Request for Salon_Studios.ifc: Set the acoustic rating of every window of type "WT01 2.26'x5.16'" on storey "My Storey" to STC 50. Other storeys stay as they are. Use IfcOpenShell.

First a look at what the model holds.

```python
import ifcopenshell
import ifcopenshell.util.element

model = ifcopenshell.open("Salon_Studios.ifc")
print(model.schema)
storey = next(s for s in model.by_type("IfcBuildingStorey") if s.Name == "My Storey")
windows = [e for e in ifcopenshell.util.element.get_decomposition(storey) if e.is_a("IfcWindow")]
seen = {}
for e in windows:
    element_type = ifcopenshell.util.element.get_type(e)
    key = (element_type.Name if element_type != e and element_type else None, ifcopenshell.util.element.get_pset(e, "Pset_WindowCommon", "AcousticRating"))
    seen[key] = seen.get(key, 0) + 1
for (name, value), count in sorted(seen.items(), key=str):
    print(count, "x", name, "|", value)
```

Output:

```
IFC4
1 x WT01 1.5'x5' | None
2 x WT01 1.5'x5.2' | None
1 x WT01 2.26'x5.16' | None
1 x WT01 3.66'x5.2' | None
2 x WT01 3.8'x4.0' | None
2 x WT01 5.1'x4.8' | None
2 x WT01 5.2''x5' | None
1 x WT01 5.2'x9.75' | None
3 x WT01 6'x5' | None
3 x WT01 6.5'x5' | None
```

```python
import ifcopenshell
import ifcopenshell.api.pset
import ifcopenshell.util.element

model = ifcopenshell.open("Salon_Studios.ifc")

storey = next(s for s in model.by_type("IfcBuildingStorey") if s.Name == "My Storey")
windows = [e for e in ifcopenshell.util.element.get_decomposition(storey) if e.is_a("IfcWindow")]

count = 0
for e in windows:
    element_type = ifcopenshell.util.element.get_type(e)
    if element_type in (None, e) or element_type.Name != "WT01 2.26'x5.16'":
        continue
    # add_pset returns the element's existing set when there is one.
    pset = ifcopenshell.api.pset.add_pset(model, product=e, name="Pset_WindowCommon")
    ifcopenshell.api.pset.edit_pset(model, pset=pset, properties={"AcousticRating": "STC 50"})
    count += 1

print(count, "windows updated")

model.write("Salon_Studios_edited.ifc")
```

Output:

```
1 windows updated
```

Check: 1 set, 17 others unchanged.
